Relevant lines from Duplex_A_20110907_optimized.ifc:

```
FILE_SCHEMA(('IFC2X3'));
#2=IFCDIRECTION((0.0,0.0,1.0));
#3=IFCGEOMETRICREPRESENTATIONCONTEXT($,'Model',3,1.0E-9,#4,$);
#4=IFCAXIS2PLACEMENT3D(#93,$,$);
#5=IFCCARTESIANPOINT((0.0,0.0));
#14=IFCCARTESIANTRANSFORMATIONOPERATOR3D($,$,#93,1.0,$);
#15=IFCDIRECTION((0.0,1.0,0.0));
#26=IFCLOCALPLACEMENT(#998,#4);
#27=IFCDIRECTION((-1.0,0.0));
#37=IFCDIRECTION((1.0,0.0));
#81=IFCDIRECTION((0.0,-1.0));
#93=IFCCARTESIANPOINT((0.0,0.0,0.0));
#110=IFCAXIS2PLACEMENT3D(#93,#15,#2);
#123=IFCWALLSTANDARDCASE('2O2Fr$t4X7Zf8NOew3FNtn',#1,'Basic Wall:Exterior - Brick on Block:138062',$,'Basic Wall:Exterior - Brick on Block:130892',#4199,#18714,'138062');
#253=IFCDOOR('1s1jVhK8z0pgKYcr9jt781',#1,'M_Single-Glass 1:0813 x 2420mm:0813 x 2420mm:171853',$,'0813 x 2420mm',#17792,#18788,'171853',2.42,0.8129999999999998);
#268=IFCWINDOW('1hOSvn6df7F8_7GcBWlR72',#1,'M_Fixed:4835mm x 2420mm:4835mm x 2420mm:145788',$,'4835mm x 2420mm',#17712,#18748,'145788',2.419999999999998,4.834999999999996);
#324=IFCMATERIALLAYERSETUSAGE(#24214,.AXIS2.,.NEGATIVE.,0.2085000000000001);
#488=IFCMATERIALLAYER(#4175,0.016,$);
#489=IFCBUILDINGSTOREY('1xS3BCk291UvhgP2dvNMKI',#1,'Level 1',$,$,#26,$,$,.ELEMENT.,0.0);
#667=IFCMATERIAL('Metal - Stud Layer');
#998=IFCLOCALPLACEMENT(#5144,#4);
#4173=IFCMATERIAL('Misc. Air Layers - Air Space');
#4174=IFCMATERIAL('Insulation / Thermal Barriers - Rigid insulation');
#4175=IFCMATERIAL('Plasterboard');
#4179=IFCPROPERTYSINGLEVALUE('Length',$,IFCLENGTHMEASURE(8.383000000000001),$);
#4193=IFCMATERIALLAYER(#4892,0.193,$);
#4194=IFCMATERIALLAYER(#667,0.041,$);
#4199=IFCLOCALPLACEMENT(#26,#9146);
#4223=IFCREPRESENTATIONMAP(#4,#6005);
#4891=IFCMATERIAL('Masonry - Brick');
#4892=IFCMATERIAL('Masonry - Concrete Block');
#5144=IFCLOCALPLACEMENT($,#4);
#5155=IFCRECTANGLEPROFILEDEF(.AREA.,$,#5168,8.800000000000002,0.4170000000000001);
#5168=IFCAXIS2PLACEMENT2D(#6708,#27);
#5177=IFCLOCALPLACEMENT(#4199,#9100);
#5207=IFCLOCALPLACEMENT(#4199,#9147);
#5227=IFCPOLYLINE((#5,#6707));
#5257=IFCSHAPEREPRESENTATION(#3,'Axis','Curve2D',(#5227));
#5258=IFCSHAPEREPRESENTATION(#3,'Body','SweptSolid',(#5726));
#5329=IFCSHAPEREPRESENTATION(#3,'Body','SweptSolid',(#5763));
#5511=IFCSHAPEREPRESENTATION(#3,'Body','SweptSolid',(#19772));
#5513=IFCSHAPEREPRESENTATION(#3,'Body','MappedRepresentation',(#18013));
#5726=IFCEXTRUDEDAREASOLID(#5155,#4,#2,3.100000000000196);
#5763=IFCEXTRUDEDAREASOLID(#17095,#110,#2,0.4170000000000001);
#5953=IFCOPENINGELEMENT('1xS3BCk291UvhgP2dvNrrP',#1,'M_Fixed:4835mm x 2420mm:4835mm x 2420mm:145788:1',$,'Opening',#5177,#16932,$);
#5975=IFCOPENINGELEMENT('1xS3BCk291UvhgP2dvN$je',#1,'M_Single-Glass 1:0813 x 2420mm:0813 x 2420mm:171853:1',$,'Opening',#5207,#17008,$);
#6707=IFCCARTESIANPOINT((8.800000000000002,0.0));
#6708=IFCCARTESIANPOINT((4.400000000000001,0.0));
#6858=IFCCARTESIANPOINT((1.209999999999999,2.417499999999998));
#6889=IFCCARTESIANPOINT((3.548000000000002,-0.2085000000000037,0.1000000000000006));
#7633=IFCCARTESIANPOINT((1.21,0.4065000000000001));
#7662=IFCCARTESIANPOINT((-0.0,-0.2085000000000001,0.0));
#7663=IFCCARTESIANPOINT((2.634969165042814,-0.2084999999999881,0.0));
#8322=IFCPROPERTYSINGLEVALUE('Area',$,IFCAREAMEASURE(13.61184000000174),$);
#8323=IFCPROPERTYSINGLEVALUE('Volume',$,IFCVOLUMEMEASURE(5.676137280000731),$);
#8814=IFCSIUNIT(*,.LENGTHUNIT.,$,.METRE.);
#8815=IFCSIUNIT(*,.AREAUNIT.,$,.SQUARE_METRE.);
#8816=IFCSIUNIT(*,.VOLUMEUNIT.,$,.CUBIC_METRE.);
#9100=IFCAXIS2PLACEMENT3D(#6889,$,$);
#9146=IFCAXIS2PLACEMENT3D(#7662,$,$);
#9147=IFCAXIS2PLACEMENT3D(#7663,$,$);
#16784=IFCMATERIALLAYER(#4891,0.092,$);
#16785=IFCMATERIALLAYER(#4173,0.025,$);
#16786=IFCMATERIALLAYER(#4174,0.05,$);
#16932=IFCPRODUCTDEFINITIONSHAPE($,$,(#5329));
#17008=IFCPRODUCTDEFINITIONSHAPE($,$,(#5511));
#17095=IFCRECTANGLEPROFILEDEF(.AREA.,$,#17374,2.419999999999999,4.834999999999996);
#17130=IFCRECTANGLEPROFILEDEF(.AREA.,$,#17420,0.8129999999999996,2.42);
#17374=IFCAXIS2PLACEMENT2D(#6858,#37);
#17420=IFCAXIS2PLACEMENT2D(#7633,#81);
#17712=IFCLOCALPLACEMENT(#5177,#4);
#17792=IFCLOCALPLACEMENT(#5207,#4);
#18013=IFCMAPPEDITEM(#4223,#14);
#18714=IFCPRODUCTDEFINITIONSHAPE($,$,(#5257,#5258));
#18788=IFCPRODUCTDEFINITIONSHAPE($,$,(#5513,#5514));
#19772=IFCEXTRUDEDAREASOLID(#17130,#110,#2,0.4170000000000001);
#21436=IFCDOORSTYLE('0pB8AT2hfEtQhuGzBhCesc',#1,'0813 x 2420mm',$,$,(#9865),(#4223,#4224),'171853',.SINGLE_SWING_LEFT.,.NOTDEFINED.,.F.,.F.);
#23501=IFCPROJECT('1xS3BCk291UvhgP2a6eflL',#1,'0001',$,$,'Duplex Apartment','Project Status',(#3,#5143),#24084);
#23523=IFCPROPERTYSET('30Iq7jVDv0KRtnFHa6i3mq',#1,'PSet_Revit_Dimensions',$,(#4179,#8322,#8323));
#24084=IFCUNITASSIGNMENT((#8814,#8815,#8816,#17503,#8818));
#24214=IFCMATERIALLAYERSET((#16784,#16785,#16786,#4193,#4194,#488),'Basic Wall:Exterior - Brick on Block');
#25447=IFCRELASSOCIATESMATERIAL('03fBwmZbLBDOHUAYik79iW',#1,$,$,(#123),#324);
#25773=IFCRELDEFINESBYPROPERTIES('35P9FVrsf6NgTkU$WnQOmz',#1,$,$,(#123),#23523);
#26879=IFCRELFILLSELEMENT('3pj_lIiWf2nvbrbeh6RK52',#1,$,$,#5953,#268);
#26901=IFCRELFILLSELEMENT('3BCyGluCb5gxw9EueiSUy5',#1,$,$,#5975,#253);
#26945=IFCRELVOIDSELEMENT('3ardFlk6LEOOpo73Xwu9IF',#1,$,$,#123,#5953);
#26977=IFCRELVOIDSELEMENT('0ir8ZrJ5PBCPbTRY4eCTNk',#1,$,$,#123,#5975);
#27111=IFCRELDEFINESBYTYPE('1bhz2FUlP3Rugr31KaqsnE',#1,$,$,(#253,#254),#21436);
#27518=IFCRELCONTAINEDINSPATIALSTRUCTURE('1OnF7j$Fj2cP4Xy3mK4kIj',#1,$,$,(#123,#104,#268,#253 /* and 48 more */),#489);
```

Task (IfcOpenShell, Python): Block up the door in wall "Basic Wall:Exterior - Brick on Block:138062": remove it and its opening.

```python
import ifcopenshell
import ifcopenshell.api.feature
import ifcopenshell.api.pset
import ifcopenshell.api.root
import ifcopenshell.geom
import ifcopenshell.util.element
import ifcopenshell.util.shape
import ifcopenshell.util.unit

model = ifcopenshell.open("Duplex_A_20110907_optimized.ifc")
area_scale = ifcopenshell.util.unit.calculate_unit_scale(model, "AREAUNIT")
volume_scale = ifcopenshell.util.unit.calculate_unit_scale(model, "VOLUMEUNIT")
settings = ifcopenshell.geom.settings()


def volume(element):
    """Net volume in cubic metres, openings subtracted."""
    shape = ifcopenshell.geom.create_shape(settings, element)
    return ifcopenshell.util.shape.get_volume(shape.geometry)


door = model.by_guid("1s1jVhK8z0pgKYcr9jt781")
opening = door.FillsVoids[0].RelatingOpeningElement
wall = opening.VoidsElements[0].RelatingBuildingElement
before = volume(wall)

ifcopenshell.api.root.remove_product(model, product=door)
ifcopenshell.api.feature.remove_feature(model, feature=opening)

after = volume(wall)
thickness = 0.417  # wall thickness in metres

# Update the wall's stored quantities.
pset = model.by_id(ifcopenshell.util.element.get_pset(wall, "PSet_Revit_Dimensions", should_inherit=False)["id"])
ifcopenshell.api.pset.edit_pset(model, pset=pset, properties={
    "Area": model.create_entity("IfcAreaMeasure", after / thickness / area_scale),
    "Volume": model.create_entity("IfcVolumeMeasure", after / volume_scale),
})

print(f"wall volume {before:.3f} -> {after:.3f} m3")

model.write("Duplex_A_20110907_optimized_updated.ifc")
```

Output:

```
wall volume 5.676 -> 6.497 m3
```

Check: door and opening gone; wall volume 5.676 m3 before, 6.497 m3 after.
